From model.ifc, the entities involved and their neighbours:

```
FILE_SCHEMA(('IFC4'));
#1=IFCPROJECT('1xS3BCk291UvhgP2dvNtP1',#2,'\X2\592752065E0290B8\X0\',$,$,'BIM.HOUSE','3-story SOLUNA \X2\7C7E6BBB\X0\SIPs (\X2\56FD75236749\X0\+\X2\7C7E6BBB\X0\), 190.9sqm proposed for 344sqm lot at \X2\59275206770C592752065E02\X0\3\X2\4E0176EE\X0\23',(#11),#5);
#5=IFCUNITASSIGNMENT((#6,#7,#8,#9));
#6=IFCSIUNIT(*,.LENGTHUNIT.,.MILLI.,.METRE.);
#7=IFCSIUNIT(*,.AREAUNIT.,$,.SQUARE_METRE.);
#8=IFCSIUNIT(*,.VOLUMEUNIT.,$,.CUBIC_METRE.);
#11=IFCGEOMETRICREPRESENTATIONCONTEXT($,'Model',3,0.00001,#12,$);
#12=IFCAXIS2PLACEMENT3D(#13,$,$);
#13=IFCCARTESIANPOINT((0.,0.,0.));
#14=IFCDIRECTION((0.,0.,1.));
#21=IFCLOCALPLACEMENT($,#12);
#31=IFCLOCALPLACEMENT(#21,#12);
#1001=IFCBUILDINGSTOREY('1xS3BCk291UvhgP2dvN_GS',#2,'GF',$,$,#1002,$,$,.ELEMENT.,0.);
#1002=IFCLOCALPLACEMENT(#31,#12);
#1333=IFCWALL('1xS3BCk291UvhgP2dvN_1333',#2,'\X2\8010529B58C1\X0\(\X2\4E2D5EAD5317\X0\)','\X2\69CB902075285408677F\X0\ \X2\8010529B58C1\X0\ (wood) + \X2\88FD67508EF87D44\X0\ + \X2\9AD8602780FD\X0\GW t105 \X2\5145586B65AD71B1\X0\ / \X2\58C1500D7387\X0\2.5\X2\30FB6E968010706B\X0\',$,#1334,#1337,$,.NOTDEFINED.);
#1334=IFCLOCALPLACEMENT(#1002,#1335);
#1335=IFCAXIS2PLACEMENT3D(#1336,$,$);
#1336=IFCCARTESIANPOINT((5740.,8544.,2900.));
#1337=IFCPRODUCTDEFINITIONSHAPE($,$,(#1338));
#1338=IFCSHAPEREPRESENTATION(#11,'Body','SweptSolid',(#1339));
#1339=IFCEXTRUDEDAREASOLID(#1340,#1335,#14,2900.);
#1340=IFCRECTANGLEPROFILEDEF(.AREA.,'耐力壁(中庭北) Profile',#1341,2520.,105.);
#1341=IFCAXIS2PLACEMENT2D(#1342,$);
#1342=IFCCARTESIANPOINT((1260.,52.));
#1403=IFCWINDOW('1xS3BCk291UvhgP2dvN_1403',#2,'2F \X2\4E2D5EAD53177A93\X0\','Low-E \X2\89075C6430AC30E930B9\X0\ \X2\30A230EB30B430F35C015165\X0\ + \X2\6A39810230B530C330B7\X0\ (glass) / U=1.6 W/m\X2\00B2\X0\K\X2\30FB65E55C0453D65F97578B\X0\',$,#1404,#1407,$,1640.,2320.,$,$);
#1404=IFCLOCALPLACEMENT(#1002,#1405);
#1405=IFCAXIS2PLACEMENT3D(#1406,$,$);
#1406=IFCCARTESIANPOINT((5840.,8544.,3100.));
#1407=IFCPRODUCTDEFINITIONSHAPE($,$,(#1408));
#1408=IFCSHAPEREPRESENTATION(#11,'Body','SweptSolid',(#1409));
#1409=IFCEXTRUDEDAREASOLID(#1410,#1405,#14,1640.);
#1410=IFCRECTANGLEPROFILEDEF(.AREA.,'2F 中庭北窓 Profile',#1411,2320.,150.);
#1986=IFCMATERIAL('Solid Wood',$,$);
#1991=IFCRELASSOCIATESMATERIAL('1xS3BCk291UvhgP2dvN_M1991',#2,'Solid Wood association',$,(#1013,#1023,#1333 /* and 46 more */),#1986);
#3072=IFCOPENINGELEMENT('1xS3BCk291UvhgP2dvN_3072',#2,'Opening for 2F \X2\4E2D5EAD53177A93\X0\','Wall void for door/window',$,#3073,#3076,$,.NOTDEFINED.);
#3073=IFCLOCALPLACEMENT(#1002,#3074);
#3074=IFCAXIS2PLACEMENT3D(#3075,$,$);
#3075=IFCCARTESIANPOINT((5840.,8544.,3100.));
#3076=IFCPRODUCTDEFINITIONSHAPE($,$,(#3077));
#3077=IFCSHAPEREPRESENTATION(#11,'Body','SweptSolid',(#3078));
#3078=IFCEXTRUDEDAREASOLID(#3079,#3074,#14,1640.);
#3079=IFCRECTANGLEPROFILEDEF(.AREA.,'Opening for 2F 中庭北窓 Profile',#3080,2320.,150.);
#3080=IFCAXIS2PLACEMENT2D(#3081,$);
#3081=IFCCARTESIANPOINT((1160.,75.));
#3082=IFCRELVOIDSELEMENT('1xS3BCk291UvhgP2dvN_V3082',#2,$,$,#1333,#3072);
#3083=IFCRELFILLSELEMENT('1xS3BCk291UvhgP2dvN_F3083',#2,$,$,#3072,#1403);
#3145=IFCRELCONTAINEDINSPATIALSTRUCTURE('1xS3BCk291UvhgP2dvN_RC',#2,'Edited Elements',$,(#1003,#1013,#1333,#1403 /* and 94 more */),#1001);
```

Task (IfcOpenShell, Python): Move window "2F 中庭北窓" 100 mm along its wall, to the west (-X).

```python
import ifcopenshell
import ifcopenshell.api.geometry
import ifcopenshell.util.placement
import ifcopenshell.util.unit

model = ifcopenshell.open("model.ifc")
unit_scale = ifcopenshell.util.unit.calculate_unit_scale(model)

window = model.by_guid("1xS3BCk291UvhgP2dvN_1403")
opening = window.FillsVoids[0].RelatingOpeningElement
wall = opening.VoidsElements[0].RelatingBuildingElement

wall_matrix = ifcopenshell.util.placement.get_local_placement(wall.ObjectPlacement)
shift = wall_matrix[:3, 0] * -0.1 / unit_scale
before = ifcopenshell.util.placement.get_local_placement(window.ObjectPlacement)[:3, 3].copy()

# The window is not placed relative to its opening, so move both.
for product in (opening, window):
    matrix = ifcopenshell.util.placement.get_local_placement(product.ObjectPlacement)
    matrix[:3, 3] += shift
    ifcopenshell.api.geometry.edit_object_placement(model, product=product, matrix=matrix, is_si=False)

after = ifcopenshell.util.placement.get_local_placement(window.ObjectPlacement)[:3, 3]
print("window moved by", (after - before).round(3) + 0.0)

model.write("model_updated.ifc")
```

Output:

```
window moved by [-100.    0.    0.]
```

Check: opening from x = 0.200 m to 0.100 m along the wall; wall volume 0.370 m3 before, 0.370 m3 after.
